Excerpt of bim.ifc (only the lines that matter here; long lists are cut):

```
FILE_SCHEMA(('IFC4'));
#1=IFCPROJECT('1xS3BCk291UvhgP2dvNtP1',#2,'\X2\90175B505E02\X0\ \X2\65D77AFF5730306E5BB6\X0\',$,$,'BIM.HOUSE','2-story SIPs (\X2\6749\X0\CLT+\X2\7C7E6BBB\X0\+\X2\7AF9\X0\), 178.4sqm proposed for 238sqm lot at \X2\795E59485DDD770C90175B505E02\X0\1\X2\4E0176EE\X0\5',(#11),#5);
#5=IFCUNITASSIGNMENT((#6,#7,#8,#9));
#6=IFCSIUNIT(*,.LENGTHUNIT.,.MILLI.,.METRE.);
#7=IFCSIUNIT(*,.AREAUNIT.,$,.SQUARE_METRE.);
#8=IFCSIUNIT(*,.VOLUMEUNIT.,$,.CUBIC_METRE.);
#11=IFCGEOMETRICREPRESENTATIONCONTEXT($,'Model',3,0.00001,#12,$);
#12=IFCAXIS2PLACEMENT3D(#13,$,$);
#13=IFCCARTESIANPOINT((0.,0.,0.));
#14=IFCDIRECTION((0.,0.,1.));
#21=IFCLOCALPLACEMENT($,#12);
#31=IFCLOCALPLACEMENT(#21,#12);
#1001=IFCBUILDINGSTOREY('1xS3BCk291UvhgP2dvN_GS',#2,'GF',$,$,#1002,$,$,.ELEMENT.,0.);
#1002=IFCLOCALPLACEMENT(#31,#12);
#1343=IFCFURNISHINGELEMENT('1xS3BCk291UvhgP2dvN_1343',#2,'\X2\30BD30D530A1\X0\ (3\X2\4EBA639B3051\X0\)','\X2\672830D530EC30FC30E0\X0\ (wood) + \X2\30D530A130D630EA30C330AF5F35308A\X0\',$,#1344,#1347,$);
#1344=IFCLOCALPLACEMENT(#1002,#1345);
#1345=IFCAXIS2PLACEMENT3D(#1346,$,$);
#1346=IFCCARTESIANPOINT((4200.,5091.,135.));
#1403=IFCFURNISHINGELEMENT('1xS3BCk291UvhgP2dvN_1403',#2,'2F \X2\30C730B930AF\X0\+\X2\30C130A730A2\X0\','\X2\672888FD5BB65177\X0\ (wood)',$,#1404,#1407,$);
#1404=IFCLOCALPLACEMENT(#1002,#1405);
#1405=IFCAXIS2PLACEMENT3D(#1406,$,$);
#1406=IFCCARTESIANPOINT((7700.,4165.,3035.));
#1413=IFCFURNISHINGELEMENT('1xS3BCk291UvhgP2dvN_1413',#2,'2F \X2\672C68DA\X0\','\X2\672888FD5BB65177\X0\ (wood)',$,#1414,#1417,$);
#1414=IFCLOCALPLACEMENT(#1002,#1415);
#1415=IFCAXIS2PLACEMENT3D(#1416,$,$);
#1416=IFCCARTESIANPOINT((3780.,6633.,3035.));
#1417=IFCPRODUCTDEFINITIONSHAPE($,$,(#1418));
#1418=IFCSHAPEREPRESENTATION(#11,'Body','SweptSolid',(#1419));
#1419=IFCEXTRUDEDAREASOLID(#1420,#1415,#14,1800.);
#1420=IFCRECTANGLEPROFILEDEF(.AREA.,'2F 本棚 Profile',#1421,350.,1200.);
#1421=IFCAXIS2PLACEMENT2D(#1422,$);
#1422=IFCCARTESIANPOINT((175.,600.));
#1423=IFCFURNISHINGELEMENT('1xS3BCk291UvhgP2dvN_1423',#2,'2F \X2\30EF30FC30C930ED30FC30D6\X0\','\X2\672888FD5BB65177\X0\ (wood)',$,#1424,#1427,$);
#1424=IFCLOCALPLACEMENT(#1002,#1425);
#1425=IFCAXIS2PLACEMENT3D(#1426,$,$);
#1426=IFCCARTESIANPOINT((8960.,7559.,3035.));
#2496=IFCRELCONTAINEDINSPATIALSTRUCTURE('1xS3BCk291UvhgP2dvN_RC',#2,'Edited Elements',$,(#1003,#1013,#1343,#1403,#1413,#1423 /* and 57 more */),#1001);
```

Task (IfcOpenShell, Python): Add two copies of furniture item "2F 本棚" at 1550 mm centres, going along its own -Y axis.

```python
import ifcopenshell
import ifcopenshell.api.geometry
import ifcopenshell.api.root
import ifcopenshell.util.element
import ifcopenshell.util.placement
import ifcopenshell.util.unit

model = ifcopenshell.open("bim.ifc")
unit_scale = ifcopenshell.util.unit.calculate_unit_scale(model)


def reuse_history(source, copy):
    """copy_class also copies each property set's owner history, people and application; keep the originals."""
    for rel in copy.IsDefinedBy:
        if rel.is_a("IfcRelDefinesByProperties") and (history := rel.RelatingPropertyDefinition.OwnerHistory):
            rel.RelatingPropertyDefinition.OwnerHistory = source.OwnerHistory
            ifcopenshell.util.element.remove_deep2(model, history)


source = model.by_id(1413)
base = ifcopenshell.util.placement.get_local_placement(source.ObjectPlacement)
step = -base[:3, 1] * 1.55 / unit_scale

for i in range(1, 3):
    copy = ifcopenshell.api.root.copy_class(model, product=source)
    copy.Representation = ifcopenshell.util.element.copy_deep(
        model, source.Representation, exclude=["IfcGeometricRepresentationContext", "IfcRepresentationMap"]
    )
    reuse_history(source, copy)
    matrix = base.copy()
    matrix[:3, 3] += i * step
    print("added at", matrix[:3, 3].round(3) + 0.0)
    ifcopenshell.api.geometry.edit_object_placement(model, product=copy, matrix=matrix, is_si=False)

model.write("bim-out.ifc")
```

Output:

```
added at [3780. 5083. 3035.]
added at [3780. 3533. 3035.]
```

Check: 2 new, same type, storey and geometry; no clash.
